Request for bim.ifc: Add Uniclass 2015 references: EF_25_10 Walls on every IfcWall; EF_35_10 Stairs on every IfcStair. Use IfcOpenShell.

First a look at what the model holds.

```python
import ifcopenshell

model = ifcopenshell.open("bim.ifc")
print(model.schema)
print("classifications:", [c.Name for c in model.by_type("IfcClassification")])
for ifc_class in ("IfcDoor", "IfcRoof", "IfcStair", "IfcWall", "IfcWindow"):
    print(ifc_class, len(model.by_type(ifc_class)))
```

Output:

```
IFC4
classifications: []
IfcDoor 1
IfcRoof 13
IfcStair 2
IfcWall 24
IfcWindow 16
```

```python
import ifcopenshell
import ifcopenshell.api.classification

model = ifcopenshell.open("bim.ifc")

system = ifcopenshell.api.classification.add_classification(model, classification="Uniclass 2015")

codes = {
    "IfcWall": ("EF_25_10", "Walls"),
    "IfcStair": ("EF_35_10", "Stairs"),
}
for ifc_class, (code, name) in codes.items():
    products = model.by_type(ifc_class)
    ifcopenshell.api.classification.add_reference(
        model, products=products, classification=system, identification=code, name=name
    )
    print(code, len(products))

model.write("bim_v2.ifc")
```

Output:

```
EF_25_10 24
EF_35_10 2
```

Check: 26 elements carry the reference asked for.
